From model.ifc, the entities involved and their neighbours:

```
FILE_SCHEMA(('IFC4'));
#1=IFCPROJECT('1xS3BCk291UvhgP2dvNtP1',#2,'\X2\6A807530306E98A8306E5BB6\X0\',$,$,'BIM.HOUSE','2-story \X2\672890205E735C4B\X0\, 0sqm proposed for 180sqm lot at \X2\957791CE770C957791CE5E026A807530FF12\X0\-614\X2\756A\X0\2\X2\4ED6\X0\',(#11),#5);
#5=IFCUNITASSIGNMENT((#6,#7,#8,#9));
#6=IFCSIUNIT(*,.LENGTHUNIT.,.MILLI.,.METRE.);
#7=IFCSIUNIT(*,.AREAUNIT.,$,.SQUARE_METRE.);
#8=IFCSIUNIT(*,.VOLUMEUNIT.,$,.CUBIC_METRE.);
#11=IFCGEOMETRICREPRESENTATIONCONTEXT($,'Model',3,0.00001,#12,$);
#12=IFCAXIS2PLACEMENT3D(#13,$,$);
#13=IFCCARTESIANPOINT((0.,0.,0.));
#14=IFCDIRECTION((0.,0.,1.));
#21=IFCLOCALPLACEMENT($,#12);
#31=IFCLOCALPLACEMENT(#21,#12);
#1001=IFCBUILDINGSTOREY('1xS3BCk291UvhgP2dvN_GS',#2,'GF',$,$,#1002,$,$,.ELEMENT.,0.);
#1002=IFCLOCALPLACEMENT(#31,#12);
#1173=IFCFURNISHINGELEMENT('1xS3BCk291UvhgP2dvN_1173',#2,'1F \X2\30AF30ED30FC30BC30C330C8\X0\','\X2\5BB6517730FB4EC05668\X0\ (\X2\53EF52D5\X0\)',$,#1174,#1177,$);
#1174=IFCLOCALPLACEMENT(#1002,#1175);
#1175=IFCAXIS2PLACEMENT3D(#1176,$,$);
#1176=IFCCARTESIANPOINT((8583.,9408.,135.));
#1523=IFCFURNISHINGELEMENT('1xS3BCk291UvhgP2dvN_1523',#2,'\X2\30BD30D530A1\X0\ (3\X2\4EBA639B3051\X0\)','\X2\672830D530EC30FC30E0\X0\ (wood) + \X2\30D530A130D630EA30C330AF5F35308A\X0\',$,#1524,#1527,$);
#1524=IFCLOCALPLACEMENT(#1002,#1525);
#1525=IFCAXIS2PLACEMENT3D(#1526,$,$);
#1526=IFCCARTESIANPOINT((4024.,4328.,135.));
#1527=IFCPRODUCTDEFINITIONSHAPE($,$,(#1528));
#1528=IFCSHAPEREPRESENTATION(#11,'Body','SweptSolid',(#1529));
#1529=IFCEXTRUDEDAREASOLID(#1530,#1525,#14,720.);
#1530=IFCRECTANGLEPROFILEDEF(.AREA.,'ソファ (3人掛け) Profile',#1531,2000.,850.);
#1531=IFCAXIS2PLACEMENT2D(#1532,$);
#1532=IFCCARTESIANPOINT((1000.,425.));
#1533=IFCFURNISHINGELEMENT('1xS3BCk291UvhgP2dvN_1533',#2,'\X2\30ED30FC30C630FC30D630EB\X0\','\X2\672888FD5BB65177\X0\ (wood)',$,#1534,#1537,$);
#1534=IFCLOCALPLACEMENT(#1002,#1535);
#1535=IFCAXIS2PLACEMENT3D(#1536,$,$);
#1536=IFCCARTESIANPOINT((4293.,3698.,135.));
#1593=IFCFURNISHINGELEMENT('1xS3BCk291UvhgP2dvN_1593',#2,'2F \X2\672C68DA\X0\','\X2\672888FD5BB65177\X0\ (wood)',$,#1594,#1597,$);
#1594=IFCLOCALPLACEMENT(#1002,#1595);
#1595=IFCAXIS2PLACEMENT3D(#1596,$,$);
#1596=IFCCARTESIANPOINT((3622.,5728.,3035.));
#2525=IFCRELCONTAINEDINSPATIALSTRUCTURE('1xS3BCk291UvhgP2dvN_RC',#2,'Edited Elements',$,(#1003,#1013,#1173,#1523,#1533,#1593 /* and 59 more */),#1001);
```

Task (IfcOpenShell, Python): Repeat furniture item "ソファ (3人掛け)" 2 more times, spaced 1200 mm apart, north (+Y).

```python
import numpy as np
import ifcopenshell
import ifcopenshell.api.geometry
import ifcopenshell.api.root
import ifcopenshell.util.element
import ifcopenshell.util.placement
import ifcopenshell.util.unit

model = ifcopenshell.open("model.ifc")
unit_scale = ifcopenshell.util.unit.calculate_unit_scale(model)


def reuse_history(source, copy):
    """copy_class also copies each property set's owner history, people and application; keep the originals."""
    for rel in copy.IsDefinedBy:
        if rel.is_a("IfcRelDefinesByProperties") and (history := rel.RelatingPropertyDefinition.OwnerHistory):
            rel.RelatingPropertyDefinition.OwnerHistory = source.OwnerHistory
            ifcopenshell.util.element.remove_deep2(model, history)


source = model.by_guid("1xS3BCk291UvhgP2dvN_1523")
base = ifcopenshell.util.placement.get_local_placement(source.ObjectPlacement)
step = np.array([0.0, 1.0, 0.0]) * 1.2 / unit_scale

for i in range(1, 3):
    copy = ifcopenshell.api.root.copy_class(model, product=source)
    copy.Representation = ifcopenshell.util.element.copy_deep(
        model, source.Representation, exclude=["IfcGeometricRepresentationContext", "IfcRepresentationMap"]
    )
    reuse_history(source, copy)
    matrix = base.copy()
    matrix[:3, 3] += i * step
    print("added at", matrix[:3, 3].round(3) + 0.0)
    ifcopenshell.api.geometry.edit_object_placement(model, product=copy, matrix=matrix, is_si=False)

model.write("model_v2.ifc")
```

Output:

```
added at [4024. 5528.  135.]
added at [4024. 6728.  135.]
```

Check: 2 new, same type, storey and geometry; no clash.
